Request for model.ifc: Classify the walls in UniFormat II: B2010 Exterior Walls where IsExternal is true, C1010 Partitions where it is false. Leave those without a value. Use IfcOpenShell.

First a look at what the model holds.

```python
import ifcopenshell
import ifcopenshell.util.element

model = ifcopenshell.open("model.ifc")
print(model.schema)
print("classifications:", [c.Name for c in model.by_type("IfcClassification")])
values = [ifcopenshell.util.element.get_pset(e, "Pset_WallCommon", "IsExternal") for e in model.by_type("IfcWall")]
for value in (True, False, None):
    print("IsExternal", value, values.count(value))
```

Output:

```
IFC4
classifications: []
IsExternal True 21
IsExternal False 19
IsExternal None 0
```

```python
import ifcopenshell
import ifcopenshell.api.classification
import ifcopenshell.util.element

model = ifcopenshell.open("model.ifc")

system = ifcopenshell.api.classification.add_classification(model, classification="UniFormat II")

walls = model.by_type("IfcWall")
external = {e: ifcopenshell.util.element.get_pset(e, "Pset_WallCommon", "IsExternal") for e in walls}
for flag, code, name in ((True, "B2010", "Exterior Walls"), (False, "C1010", "Partitions")):
    products = [e for e in walls if external[e] is flag]
    ifcopenshell.api.classification.add_reference(
        model, products=products, classification=system, identification=code, name=name
    )
    print(code, len(products))

model.write("model-out.ifc")
```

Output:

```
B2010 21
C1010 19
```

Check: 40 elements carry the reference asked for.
